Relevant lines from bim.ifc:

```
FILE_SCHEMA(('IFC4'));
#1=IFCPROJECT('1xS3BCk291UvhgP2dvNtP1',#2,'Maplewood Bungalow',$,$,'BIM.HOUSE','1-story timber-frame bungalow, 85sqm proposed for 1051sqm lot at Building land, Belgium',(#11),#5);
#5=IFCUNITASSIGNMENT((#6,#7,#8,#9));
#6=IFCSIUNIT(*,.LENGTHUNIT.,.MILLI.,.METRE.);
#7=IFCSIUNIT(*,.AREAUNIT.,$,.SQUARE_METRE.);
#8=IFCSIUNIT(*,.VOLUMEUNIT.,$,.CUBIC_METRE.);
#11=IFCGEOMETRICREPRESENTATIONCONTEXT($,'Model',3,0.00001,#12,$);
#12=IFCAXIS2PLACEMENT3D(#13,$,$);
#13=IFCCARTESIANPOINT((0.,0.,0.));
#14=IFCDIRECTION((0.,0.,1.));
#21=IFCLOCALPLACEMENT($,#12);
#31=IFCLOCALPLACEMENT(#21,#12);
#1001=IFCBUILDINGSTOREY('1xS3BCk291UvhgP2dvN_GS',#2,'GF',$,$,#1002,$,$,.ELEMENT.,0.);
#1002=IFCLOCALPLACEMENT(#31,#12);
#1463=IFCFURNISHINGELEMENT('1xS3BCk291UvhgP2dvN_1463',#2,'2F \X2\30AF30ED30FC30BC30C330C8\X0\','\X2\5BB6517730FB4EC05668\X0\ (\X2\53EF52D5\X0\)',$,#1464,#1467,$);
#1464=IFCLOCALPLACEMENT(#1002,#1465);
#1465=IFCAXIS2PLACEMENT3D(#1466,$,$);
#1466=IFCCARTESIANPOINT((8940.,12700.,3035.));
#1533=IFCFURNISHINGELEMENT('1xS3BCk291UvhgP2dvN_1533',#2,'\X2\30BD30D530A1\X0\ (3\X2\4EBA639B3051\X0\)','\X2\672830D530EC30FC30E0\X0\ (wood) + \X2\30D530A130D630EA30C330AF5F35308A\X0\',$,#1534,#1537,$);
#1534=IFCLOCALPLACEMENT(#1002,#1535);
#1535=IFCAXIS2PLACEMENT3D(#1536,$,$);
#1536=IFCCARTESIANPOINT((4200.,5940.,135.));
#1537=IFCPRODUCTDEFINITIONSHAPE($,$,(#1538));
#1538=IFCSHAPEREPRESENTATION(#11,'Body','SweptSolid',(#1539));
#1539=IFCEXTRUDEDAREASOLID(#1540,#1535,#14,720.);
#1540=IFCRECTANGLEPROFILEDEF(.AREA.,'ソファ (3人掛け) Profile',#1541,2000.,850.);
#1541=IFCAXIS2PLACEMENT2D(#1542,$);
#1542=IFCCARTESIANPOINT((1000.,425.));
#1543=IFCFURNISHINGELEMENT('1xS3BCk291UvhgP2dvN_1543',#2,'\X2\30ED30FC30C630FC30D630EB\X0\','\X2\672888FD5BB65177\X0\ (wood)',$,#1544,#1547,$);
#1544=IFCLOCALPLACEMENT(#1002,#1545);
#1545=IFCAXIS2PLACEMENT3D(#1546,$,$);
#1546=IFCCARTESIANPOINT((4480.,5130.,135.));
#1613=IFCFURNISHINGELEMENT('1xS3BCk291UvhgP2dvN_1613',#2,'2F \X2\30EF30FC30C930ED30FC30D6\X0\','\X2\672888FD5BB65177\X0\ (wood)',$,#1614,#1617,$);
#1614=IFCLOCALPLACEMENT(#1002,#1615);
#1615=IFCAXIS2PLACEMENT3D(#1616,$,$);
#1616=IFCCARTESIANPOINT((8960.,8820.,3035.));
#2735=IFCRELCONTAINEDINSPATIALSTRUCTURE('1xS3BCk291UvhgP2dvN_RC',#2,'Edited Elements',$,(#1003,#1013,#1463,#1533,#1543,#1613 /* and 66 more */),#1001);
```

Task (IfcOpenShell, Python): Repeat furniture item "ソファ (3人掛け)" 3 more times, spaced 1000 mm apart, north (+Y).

```python
import numpy as np
import ifcopenshell
import ifcopenshell.api.geometry
import ifcopenshell.api.root
import ifcopenshell.util.element
import ifcopenshell.util.placement

model = ifcopenshell.open("bim.ifc")


def reuse_history(source, copy):
    """copy_class also copies each property set's owner history, people and application; keep the originals."""
    for rel in copy.IsDefinedBy:
        if rel.is_a("IfcRelDefinesByProperties") and (history := rel.RelatingPropertyDefinition.OwnerHistory):
            rel.RelatingPropertyDefinition.OwnerHistory = source.OwnerHistory
            ifcopenshell.util.element.remove_deep2(model, history)


source = model.by_id(1533)
base = ifcopenshell.util.placement.get_local_placement(source.ObjectPlacement)
step = np.array([0.0, 1.0, 0.0]) * 1000.0

for i in range(1, 4):
    copy = ifcopenshell.api.root.copy_class(model, product=source)
    copy.Representation = ifcopenshell.util.element.copy_deep(
        model, source.Representation, exclude=["IfcGeometricRepresentationContext", "IfcRepresentationMap"]
    )
    reuse_history(source, copy)
    matrix = base.copy()
    matrix[:3, 3] += i * step
    print("added at", matrix[:3, 3].round(3) + 0.0)
    ifcopenshell.api.geometry.edit_object_placement(model, product=copy, matrix=matrix, is_si=False)

model.write("bim_edited.ifc")
```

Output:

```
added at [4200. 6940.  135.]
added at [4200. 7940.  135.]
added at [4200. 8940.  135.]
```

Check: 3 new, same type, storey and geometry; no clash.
